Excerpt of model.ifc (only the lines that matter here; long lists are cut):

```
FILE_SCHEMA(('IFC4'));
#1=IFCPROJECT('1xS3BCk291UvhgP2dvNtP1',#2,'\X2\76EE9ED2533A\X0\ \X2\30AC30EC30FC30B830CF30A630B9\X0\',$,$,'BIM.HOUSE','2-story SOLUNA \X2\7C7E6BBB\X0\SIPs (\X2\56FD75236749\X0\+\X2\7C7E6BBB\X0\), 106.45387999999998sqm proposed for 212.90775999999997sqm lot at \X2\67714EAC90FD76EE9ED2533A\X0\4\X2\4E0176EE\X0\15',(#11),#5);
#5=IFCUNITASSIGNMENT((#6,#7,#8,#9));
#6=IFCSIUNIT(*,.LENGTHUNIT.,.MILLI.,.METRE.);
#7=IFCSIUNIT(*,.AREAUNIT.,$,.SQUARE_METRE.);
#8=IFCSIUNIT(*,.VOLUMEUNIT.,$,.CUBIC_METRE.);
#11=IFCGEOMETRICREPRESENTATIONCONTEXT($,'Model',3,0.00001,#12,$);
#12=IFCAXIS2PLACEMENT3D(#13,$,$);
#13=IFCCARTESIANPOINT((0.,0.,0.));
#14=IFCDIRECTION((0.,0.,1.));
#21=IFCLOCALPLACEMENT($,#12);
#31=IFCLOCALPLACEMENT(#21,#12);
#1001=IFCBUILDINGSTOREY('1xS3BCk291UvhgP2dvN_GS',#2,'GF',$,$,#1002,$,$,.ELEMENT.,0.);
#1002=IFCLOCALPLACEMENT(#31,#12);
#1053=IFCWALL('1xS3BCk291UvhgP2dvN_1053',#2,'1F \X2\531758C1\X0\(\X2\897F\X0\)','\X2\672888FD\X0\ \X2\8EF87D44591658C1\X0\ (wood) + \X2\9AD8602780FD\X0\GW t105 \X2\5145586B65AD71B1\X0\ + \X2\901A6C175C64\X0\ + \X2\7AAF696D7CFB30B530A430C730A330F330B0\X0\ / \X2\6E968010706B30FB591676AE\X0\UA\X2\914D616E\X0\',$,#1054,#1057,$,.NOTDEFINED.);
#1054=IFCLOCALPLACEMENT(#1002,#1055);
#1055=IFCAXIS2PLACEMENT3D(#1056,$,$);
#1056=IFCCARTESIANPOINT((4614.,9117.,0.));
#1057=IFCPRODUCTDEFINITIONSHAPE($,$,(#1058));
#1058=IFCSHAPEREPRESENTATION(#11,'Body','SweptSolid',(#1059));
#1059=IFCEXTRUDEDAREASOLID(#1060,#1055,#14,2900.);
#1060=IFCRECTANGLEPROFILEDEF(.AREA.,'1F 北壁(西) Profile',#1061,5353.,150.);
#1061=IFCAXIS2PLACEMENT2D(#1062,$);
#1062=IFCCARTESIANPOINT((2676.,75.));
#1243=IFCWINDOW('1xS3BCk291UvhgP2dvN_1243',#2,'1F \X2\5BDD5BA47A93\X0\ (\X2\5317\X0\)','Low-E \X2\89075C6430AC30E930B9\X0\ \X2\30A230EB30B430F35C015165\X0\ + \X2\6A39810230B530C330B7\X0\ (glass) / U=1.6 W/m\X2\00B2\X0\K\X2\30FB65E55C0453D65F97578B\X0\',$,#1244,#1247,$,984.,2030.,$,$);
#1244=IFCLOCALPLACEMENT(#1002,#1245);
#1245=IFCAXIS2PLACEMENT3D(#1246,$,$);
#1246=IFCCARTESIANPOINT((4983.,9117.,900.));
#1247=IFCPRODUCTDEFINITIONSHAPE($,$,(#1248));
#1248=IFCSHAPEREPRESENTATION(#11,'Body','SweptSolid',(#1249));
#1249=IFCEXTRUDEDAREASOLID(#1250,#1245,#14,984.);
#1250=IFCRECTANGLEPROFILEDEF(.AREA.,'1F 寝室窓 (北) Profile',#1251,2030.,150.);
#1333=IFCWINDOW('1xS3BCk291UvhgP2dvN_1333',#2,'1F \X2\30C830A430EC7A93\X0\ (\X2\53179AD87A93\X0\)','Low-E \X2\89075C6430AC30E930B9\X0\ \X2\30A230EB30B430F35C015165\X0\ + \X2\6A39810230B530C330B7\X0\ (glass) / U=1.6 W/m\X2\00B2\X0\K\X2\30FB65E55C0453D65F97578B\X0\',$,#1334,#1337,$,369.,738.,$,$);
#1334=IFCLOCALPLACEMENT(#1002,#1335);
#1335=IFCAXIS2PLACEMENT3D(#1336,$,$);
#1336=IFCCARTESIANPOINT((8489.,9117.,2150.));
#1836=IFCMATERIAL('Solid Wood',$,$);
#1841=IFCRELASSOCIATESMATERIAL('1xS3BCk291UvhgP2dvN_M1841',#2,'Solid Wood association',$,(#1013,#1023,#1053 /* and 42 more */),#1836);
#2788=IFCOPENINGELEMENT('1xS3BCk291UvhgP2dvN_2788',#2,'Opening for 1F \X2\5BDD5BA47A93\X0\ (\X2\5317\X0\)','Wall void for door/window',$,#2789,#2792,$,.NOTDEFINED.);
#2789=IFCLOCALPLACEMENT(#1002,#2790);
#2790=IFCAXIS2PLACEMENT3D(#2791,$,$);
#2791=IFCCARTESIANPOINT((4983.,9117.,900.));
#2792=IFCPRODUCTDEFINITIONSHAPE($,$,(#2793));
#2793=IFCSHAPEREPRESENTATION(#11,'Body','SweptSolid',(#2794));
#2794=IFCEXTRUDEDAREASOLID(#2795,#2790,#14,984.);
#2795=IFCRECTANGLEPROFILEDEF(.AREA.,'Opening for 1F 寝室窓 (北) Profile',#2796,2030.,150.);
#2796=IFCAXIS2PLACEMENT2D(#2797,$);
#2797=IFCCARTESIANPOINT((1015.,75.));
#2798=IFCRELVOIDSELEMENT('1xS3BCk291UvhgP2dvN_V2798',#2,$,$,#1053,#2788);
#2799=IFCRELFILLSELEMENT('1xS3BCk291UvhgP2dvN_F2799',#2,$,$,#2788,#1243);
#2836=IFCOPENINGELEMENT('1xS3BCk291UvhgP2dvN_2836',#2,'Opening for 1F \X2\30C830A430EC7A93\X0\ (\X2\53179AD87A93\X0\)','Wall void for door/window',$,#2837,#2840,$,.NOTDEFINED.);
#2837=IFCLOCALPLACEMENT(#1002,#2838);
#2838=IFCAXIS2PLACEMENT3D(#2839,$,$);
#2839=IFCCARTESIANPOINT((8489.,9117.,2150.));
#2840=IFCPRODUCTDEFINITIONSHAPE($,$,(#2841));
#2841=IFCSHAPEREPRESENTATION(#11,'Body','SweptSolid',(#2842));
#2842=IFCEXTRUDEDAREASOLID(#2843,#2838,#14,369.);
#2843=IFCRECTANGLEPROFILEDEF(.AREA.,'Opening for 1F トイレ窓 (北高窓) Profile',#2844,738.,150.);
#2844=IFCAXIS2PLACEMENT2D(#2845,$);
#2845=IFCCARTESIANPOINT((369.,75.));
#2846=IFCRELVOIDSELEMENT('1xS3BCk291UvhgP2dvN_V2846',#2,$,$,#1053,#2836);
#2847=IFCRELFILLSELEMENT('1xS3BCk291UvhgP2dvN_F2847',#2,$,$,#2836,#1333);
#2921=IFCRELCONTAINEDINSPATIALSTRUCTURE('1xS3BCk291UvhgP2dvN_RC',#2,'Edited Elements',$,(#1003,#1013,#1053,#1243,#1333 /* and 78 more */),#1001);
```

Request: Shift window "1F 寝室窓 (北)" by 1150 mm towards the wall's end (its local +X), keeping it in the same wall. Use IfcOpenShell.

```python
import ifcopenshell
import ifcopenshell.api.geometry
import ifcopenshell.util.placement

model = ifcopenshell.open("model.ifc")

window = model.by_guid("1xS3BCk291UvhgP2dvN_1243")
opening = window.FillsVoids[0].RelatingOpeningElement
wall = opening.VoidsElements[0].RelatingBuildingElement

wall_matrix = ifcopenshell.util.placement.get_local_placement(wall.ObjectPlacement)
shift = wall_matrix[:3, 0] * 1150.0
before = ifcopenshell.util.placement.get_local_placement(window.ObjectPlacement)[:3, 3].copy()

# The window is not placed relative to its opening, so move both.
for product in (opening, window):
    matrix = ifcopenshell.util.placement.get_local_placement(product.ObjectPlacement)
    matrix[:3, 3] += shift
    ifcopenshell.api.geometry.edit_object_placement(model, product=product, matrix=matrix, is_si=False)

after = ifcopenshell.util.placement.get_local_placement(window.ObjectPlacement)[:3, 3]
print("window moved by", (after - before).round(3) + 0.0)

model.write("model_v2.ifc")
```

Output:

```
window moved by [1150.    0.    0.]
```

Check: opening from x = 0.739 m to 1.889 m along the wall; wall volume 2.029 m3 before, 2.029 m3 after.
